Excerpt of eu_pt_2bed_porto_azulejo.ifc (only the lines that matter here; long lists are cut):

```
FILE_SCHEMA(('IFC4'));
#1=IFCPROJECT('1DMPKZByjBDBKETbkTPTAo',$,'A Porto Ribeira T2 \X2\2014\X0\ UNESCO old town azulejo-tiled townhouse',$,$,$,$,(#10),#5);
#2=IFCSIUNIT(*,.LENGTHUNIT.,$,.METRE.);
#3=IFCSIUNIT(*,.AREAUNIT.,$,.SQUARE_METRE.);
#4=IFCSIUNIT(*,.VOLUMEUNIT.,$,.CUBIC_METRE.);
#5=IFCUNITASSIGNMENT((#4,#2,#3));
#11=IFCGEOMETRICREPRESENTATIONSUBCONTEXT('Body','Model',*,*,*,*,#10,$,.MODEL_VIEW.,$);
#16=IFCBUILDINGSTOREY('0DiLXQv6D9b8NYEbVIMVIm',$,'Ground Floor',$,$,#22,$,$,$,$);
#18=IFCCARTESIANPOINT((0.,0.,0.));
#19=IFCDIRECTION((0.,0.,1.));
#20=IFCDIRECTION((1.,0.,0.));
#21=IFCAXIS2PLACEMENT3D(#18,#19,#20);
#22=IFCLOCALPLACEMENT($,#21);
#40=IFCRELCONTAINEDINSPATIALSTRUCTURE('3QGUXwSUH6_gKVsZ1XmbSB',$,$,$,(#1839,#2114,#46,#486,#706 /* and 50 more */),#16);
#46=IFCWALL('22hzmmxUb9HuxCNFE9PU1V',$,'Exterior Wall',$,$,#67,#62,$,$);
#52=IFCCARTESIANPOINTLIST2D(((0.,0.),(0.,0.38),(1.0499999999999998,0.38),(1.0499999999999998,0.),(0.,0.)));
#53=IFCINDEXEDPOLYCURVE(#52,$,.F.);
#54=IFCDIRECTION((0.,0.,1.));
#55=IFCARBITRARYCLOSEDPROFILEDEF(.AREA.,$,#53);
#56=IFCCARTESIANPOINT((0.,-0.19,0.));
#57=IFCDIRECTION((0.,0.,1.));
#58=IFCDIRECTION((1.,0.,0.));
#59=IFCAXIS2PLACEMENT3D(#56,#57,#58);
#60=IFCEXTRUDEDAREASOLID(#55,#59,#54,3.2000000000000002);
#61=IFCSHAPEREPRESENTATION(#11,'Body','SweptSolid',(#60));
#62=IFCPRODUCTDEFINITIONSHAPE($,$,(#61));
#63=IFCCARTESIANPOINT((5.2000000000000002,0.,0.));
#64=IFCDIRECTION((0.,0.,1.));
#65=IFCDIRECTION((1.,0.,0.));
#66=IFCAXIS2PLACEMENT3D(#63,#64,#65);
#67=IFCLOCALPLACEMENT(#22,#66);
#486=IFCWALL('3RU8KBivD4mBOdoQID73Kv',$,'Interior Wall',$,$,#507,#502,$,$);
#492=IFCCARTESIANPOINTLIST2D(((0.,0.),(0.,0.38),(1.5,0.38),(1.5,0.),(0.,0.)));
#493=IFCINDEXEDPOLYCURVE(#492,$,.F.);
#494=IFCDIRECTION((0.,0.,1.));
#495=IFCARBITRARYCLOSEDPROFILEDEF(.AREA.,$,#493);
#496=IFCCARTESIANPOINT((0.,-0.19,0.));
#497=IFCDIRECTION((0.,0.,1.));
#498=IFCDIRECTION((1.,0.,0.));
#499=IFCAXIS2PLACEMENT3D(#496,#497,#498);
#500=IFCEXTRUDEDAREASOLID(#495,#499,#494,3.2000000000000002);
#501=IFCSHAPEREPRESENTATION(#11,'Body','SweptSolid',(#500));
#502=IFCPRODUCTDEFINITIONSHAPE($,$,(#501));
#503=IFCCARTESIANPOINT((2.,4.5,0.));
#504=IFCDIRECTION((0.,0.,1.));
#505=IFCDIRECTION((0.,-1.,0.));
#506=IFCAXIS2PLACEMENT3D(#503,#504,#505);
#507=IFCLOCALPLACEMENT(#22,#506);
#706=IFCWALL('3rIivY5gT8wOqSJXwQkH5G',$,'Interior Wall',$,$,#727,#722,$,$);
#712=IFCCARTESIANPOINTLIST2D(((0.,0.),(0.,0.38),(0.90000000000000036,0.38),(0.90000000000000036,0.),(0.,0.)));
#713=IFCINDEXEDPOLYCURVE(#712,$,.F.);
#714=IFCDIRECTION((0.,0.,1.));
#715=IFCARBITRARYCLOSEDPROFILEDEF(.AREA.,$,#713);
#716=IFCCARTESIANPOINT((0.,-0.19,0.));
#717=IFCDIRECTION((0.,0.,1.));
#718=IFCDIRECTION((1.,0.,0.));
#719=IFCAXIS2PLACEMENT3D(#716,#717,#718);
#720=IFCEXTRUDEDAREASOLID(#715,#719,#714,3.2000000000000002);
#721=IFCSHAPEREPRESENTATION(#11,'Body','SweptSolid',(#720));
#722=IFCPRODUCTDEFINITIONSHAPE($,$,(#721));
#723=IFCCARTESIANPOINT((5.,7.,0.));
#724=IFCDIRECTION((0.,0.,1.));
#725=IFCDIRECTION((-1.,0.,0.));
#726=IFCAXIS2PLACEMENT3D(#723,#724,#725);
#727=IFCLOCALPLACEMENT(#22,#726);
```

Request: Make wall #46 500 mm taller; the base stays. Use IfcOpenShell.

```python
import ifcopenshell
import ifcopenshell.geom
import ifcopenshell.util.representation
import ifcopenshell.util.shape

model = ifcopenshell.open("eu_pt_2bed_porto_azulejo.ifc")
settings = ifcopenshell.geom.settings()


def volume(element):
    """Net volume in cubic metres, openings subtracted."""
    shape = ifcopenshell.geom.create_shape(settings, element)
    return ifcopenshell.util.shape.get_volume(shape.geometry)


wall = model.by_guid("22hzmmxUb9HuxCNFE9PU1V")
before = volume(wall)

body = ifcopenshell.util.representation.get_representation(wall, "Model", "Body")
solid = body.Items[0]
old_height = solid.Depth
solid.Depth += 0.5
after = volume(wall)

print(f"height {old_height:g} -> {solid.Depth:g}, volume {before:.3f} -> {after:.3f} m3")

model.write("eu_pt_2bed_porto_azulejo_updated.ifc")
```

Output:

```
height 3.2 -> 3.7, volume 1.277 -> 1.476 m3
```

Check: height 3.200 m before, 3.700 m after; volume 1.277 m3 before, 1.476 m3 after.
